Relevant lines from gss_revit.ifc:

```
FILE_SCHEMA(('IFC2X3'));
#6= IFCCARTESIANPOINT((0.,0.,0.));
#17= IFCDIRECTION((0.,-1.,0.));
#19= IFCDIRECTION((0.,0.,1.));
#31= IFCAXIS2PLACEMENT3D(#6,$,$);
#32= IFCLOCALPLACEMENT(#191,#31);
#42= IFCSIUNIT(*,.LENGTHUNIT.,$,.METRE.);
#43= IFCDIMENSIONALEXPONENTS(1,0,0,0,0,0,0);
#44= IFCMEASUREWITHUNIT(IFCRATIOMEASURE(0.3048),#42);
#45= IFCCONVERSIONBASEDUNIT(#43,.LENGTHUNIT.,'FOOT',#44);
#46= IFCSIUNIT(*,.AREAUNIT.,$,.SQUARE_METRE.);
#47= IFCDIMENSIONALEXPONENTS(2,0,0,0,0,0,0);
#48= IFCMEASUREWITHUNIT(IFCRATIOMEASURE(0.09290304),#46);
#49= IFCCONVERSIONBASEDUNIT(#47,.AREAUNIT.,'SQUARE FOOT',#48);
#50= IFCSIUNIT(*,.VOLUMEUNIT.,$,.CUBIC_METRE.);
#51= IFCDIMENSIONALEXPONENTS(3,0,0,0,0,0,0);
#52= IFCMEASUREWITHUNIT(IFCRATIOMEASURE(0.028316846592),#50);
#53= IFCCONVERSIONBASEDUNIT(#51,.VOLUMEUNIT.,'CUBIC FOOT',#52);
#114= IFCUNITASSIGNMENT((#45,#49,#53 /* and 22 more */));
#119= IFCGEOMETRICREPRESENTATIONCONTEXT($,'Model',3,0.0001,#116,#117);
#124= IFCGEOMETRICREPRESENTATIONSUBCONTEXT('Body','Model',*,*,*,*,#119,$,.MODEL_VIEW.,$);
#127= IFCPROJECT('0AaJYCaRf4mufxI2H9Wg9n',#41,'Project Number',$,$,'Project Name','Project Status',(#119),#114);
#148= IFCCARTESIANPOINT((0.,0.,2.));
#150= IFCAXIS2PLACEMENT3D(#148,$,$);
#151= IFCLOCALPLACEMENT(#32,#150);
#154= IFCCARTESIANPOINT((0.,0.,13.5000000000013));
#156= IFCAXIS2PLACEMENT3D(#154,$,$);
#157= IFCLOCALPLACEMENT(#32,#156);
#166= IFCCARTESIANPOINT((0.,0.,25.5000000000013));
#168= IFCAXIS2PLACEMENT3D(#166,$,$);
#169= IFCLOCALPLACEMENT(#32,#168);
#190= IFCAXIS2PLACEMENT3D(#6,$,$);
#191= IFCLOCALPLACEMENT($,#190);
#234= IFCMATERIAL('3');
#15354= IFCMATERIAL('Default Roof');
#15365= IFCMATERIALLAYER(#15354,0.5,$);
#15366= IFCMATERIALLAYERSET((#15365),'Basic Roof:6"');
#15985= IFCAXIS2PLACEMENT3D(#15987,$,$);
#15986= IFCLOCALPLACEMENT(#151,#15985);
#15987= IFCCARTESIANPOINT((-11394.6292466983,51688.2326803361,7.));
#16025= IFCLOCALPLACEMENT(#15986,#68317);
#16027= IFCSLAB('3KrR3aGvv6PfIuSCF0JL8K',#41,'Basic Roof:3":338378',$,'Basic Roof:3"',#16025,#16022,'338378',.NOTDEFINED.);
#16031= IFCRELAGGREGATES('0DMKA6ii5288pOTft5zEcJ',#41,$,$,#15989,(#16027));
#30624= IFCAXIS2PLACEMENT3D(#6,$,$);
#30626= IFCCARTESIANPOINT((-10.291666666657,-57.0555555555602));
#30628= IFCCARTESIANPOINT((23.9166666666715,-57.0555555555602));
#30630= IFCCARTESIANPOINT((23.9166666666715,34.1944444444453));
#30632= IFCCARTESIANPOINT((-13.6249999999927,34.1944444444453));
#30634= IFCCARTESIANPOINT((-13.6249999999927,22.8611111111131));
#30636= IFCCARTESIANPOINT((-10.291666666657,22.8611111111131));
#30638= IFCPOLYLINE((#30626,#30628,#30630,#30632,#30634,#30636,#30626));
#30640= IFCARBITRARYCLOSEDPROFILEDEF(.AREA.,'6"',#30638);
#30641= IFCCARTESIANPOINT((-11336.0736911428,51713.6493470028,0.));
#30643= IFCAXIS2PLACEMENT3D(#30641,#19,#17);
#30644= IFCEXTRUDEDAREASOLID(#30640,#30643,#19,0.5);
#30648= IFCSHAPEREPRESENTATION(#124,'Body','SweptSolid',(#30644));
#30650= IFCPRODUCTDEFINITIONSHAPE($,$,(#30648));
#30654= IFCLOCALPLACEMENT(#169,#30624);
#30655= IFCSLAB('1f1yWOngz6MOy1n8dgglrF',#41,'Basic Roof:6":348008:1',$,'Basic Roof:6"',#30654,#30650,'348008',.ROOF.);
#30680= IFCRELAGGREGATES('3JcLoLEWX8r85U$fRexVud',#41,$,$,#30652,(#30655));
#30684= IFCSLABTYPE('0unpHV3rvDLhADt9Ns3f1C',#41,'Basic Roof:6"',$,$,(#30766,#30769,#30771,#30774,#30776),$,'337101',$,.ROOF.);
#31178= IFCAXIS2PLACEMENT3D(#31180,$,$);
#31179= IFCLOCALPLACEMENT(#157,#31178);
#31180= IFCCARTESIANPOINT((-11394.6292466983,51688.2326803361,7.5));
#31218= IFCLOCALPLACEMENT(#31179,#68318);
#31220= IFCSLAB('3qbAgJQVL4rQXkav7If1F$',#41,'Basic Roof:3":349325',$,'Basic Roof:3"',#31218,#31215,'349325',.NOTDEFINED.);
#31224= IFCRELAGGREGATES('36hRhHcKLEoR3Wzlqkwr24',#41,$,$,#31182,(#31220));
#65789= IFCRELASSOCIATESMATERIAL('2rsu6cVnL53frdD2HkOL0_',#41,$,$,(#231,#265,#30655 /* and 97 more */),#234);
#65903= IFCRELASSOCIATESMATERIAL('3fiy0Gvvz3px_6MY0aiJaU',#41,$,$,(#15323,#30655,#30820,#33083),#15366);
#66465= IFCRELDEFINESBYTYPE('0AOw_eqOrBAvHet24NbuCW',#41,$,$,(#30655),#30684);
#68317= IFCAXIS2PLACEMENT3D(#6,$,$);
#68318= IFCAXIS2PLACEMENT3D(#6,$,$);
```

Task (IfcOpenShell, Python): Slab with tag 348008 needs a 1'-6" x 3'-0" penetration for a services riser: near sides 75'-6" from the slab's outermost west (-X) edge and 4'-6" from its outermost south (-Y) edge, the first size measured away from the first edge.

```python
import numpy as np
import ifcopenshell
import ifcopenshell.api.feature
import ifcopenshell.api.geometry
import ifcopenshell.api.root
import ifcopenshell.geom
import ifcopenshell.util.placement
import ifcopenshell.util.representation
import ifcopenshell.util.shape
import ifcopenshell.util.unit

model = ifcopenshell.open("gss_revit.ifc")
unit_scale = ifcopenshell.util.unit.calculate_unit_scale(model)
settings = ifcopenshell.geom.settings()


def volume(element):
    """Net volume in cubic metres, openings subtracted."""
    shape = ifcopenshell.geom.create_shape(settings, element)
    return ifcopenshell.util.shape.get_volume(shape.geometry)


slab = model.by_guid("1f1yWOngz6MOy1n8dgglrF")
before = volume(slab)

# Extent in the slab's own axes, in metres. The edges named are its -X and -Y sides.
slab_shape = ifcopenshell.geom.create_shape(settings, slab)
vertices = ifcopenshell.util.shape.get_vertices(slab_shape.geometry)
x_min, y_min, bottom = vertices.min(axis=0)
top = vertices[:, 2].max()

opening = ifcopenshell.api.root.create_entity(model, ifc_class="IfcOpeningElement", name="Services riser opening")
context = ifcopenshell.util.representation.get_context(model, "Model", "Body", "MODEL_VIEW")
width, depth = 0.4572, 0.9144
outline = [(0.0, 0.0), (width, 0.0), (width, depth), (0.0, depth), (0.0, 0.0)]
# Overshoot both faces by 50 mm so the cut is clean.
shape = ifcopenshell.api.geometry.add_slab_representation(
    model, context=context, depth=top - bottom + 0.1, polyline=outline
)
ifcopenshell.api.geometry.assign_representation(model, product=opening, representation=shape)

matrix = ifcopenshell.util.placement.get_local_placement(slab.ObjectPlacement)
matrix[:, 3] = matrix @ np.append(np.array([x_min + 23.0124, y_min + 1.3716, bottom - 0.05]) / unit_scale, 1.0)
ifcopenshell.api.geometry.edit_object_placement(model, product=opening, matrix=matrix, is_si=False)
ifcopenshell.api.feature.add_feature(model, feature=opening, element=slab)

after = volume(slab)

print(f"slab volume {before:.3f} -> {after:.3f} m3")

model.write("gss_revit-out.ifc")
```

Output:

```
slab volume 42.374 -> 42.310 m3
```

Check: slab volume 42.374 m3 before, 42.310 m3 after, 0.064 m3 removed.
